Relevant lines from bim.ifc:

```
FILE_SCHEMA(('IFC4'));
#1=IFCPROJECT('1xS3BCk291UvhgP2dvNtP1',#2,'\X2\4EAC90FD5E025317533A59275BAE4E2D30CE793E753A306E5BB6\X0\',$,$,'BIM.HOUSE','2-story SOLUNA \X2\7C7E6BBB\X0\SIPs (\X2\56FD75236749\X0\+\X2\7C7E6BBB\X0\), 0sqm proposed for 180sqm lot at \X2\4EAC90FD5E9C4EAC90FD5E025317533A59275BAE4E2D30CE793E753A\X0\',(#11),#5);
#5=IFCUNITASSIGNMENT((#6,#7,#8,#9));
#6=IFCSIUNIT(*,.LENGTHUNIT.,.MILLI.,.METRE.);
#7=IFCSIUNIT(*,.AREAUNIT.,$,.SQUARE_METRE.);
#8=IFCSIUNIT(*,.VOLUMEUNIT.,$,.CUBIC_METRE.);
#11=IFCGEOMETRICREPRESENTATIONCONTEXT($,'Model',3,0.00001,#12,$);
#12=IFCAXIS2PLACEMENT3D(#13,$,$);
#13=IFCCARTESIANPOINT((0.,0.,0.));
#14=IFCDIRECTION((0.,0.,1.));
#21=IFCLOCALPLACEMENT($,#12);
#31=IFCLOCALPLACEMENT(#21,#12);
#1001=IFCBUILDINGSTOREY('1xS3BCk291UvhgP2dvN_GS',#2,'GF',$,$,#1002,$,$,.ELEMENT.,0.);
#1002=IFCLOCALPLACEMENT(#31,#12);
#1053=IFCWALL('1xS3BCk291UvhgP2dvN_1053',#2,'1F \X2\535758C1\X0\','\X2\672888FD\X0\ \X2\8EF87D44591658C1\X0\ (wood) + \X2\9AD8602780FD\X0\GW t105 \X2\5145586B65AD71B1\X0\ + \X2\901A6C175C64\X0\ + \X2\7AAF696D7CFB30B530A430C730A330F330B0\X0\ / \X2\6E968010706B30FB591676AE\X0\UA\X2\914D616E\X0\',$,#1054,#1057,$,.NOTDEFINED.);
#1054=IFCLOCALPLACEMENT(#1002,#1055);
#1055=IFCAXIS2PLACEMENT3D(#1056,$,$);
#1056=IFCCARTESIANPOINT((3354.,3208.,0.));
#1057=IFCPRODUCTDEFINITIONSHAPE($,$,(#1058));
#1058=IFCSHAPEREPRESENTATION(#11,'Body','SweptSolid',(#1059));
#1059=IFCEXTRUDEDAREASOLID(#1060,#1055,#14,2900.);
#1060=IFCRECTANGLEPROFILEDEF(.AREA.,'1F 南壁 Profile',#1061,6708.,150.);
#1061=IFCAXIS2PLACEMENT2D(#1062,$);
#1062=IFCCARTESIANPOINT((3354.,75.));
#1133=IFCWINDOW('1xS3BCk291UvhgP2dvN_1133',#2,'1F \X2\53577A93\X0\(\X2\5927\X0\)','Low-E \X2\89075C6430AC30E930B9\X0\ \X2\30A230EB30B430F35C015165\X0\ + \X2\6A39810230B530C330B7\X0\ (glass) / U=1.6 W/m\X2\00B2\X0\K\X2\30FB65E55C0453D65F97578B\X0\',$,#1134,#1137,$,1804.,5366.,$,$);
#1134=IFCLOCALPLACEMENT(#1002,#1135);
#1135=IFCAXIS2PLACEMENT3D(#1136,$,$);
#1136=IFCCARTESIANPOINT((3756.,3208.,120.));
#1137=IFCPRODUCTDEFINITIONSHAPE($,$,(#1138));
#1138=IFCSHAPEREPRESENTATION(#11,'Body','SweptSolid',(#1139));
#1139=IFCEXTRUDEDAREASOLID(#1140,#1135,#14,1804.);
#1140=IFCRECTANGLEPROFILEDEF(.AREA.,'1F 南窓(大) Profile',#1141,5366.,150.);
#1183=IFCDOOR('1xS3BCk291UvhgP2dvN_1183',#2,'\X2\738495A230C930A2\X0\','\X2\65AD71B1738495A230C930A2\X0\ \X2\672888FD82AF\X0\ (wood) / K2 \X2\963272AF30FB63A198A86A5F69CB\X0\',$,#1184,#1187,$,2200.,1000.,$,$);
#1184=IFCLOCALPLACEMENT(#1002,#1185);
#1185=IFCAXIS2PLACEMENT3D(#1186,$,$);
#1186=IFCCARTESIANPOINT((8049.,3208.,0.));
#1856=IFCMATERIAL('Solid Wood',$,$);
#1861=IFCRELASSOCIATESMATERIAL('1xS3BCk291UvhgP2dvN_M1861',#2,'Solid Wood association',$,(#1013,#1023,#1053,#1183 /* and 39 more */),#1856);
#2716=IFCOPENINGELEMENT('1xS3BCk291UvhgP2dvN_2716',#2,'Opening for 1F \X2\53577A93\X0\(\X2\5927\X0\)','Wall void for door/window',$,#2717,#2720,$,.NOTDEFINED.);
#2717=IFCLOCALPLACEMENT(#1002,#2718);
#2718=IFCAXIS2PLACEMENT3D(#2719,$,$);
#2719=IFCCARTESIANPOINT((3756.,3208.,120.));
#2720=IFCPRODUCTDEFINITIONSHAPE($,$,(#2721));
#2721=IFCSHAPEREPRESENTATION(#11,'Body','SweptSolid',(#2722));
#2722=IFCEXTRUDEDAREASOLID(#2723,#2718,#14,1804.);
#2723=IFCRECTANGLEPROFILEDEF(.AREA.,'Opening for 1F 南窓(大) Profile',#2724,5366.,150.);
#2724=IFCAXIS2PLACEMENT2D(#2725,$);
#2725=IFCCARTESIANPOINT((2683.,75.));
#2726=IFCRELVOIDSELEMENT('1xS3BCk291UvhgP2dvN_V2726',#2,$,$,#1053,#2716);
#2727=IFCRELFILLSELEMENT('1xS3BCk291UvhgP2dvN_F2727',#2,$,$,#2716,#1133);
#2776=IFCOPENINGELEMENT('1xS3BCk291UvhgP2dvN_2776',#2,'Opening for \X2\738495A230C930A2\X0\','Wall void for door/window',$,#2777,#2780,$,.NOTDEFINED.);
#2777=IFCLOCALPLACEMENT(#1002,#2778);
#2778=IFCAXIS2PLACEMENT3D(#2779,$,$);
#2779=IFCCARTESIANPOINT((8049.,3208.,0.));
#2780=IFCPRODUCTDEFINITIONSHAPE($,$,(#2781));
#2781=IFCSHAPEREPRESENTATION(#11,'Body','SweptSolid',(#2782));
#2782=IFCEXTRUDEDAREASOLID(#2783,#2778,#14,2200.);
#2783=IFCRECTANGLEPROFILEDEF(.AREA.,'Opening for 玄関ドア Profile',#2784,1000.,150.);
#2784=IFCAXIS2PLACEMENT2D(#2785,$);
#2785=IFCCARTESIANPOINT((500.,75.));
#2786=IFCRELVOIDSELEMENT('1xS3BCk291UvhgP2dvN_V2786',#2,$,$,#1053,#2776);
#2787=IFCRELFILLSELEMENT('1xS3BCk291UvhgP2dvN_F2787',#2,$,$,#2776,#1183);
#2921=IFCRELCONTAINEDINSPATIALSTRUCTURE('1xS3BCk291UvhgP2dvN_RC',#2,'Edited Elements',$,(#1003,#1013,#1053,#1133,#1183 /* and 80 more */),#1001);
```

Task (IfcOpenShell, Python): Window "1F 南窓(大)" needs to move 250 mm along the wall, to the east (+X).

```python
import ifcopenshell
import ifcopenshell.api.geometry
import ifcopenshell.util.placement
import ifcopenshell.util.unit

model = ifcopenshell.open("bim.ifc")
unit_scale = ifcopenshell.util.unit.calculate_unit_scale(model)

window = model.by_id(1133)
opening = window.FillsVoids[0].RelatingOpeningElement
wall = opening.VoidsElements[0].RelatingBuildingElement

wall_matrix = ifcopenshell.util.placement.get_local_placement(wall.ObjectPlacement)
shift = wall_matrix[:3, 0] * 0.25 / unit_scale
before = ifcopenshell.util.placement.get_local_placement(window.ObjectPlacement)[:3, 3].copy()

# The window is not placed relative to its opening, so move both.
for product in (opening, window):
    matrix = ifcopenshell.util.placement.get_local_placement(product.ObjectPlacement)
    matrix[:3, 3] += shift
    ifcopenshell.api.geometry.edit_object_placement(model, product=product, matrix=matrix, is_si=False)

after = ifcopenshell.util.placement.get_local_placement(window.ObjectPlacement)[:3, 3]
print("window moved by", (after - before).round(3) + 0.0)

model.write("bim_edited.ifc")
```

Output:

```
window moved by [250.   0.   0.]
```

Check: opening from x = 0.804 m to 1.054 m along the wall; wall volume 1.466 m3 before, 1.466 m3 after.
